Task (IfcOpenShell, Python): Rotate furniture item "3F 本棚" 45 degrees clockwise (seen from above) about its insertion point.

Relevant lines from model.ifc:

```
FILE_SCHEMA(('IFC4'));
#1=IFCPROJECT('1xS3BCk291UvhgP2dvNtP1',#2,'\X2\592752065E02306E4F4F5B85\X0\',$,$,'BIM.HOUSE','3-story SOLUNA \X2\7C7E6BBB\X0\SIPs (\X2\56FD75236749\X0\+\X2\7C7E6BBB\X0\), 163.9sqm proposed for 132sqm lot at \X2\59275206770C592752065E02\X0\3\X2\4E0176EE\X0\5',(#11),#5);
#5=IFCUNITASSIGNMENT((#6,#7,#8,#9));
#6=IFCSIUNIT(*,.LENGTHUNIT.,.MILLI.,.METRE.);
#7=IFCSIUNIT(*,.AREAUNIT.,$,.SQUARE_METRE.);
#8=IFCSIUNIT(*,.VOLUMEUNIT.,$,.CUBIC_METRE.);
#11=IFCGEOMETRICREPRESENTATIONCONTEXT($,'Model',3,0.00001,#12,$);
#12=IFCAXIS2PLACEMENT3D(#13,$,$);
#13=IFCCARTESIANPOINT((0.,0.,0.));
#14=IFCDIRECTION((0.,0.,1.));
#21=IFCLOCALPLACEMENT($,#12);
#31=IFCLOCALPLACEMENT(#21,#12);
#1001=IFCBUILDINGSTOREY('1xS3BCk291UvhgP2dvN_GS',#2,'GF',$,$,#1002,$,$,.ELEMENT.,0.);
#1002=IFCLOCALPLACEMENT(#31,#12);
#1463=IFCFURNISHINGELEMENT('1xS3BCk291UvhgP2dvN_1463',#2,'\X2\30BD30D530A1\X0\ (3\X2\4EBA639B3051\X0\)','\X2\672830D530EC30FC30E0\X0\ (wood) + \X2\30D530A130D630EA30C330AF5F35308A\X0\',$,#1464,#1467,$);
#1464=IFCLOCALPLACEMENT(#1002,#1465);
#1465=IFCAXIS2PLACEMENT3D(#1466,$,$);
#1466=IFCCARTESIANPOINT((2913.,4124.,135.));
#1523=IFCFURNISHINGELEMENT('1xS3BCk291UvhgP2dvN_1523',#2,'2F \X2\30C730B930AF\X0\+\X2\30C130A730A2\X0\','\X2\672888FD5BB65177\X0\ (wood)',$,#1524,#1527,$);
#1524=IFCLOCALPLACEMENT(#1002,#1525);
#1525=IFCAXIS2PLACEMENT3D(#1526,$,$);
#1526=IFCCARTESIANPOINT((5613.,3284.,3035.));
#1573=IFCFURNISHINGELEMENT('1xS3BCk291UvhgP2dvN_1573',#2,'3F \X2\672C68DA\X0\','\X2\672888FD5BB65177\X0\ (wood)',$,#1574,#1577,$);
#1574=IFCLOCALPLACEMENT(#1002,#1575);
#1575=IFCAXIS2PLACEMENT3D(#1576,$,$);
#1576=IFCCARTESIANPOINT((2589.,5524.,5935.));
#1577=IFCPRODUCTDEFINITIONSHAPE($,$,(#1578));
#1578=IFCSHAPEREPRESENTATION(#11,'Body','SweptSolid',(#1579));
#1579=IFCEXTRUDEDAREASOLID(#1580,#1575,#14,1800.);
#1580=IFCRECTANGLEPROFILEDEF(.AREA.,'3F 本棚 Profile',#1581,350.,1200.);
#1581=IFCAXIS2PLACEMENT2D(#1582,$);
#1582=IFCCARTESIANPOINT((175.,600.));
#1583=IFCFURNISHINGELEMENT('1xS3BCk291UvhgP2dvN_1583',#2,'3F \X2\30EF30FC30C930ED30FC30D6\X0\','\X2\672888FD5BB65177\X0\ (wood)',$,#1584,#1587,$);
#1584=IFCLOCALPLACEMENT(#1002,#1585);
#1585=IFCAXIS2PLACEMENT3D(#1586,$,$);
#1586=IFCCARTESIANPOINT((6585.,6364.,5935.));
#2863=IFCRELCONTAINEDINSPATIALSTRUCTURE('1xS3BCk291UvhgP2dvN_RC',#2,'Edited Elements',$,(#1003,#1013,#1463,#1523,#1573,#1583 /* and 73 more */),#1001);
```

```python
import ifcopenshell
import ifcopenshell.api.geometry
import ifcopenshell.util.placement

model = ifcopenshell.open("model.ifc")

item = model.by_id(1573)
matrix = ifcopenshell.util.placement.get_local_placement(item.ObjectPlacement)
matrix = matrix @ ifcopenshell.util.placement.rotation(-45, "Z")
ifcopenshell.api.geometry.edit_object_placement(model, product=item, matrix=matrix, is_si=False)

print(ifcopenshell.util.placement.get_local_placement(item.ObjectPlacement).round(3) + 0.0)

model.write("model_updated.ifc")
```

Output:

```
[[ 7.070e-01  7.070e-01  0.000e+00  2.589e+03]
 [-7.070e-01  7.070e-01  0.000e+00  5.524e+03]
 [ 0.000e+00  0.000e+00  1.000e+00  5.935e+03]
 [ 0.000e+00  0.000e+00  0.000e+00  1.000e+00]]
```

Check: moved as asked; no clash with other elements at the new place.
